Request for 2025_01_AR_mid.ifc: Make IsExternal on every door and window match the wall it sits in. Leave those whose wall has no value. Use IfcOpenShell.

First a look at what the model holds.

```python
import ifcopenshell
import ifcopenshell.util.element

model = ifcopenshell.open("2025_01_AR_mid.ifc")
print(model.schema)
seen = {}
for e in model.by_type("IfcDoor") + model.by_type("IfcWindow"):
    if not e.FillsVoids:
        continue
    host = e.FillsVoids[0].RelatingOpeningElement.VoidsElements[0].RelatingBuildingElement
    own = ifcopenshell.util.element.get_pset(e, f"Pset_{e.is_a()[3:].removesuffix('StandardCase')}Common", "IsExternal")
    wall = ifcopenshell.util.element.get_pset(host, "Pset_WallCommon", "IsExternal")
    seen[e.is_a(), own, wall] = seen.get((e.is_a(), own, wall), 0) + 1
for (cls, own, wall), count in sorted(seen.items(), key=str):
    print(count, cls, "IsExternal:", own, "| host wall:", wall)
```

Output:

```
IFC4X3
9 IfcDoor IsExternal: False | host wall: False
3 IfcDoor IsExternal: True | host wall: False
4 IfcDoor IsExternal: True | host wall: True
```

```python
import ifcopenshell
import ifcopenshell.api.pset
import ifcopenshell.util.element

model = ifcopenshell.open("2025_01_AR_mid.ifc")

count = 0
for ifc_class, pset_name in (("IfcDoor", "Pset_DoorCommon"), ("IfcWindow", "Pset_WindowCommon")):
    for e in model.by_type(ifc_class):
        if not e.FillsVoids:
            continue
        host = e.FillsVoids[0].RelatingOpeningElement.VoidsElements[0].RelatingBuildingElement
        external = ifcopenshell.util.element.get_pset(host, "Pset_WallCommon", "IsExternal")
        if external is None or ifcopenshell.util.element.get_pset(e, pset_name, "IsExternal") == external:
            continue
        pset = ifcopenshell.api.pset.add_pset(model, product=e, name=pset_name)
        ifcopenshell.api.pset.edit_pset(model, pset=pset, properties={"IsExternal": external})
        count += 1

print(count, "updated")

model.write("2025_01_AR_mid_updated.ifc")
```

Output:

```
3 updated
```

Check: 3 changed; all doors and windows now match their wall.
